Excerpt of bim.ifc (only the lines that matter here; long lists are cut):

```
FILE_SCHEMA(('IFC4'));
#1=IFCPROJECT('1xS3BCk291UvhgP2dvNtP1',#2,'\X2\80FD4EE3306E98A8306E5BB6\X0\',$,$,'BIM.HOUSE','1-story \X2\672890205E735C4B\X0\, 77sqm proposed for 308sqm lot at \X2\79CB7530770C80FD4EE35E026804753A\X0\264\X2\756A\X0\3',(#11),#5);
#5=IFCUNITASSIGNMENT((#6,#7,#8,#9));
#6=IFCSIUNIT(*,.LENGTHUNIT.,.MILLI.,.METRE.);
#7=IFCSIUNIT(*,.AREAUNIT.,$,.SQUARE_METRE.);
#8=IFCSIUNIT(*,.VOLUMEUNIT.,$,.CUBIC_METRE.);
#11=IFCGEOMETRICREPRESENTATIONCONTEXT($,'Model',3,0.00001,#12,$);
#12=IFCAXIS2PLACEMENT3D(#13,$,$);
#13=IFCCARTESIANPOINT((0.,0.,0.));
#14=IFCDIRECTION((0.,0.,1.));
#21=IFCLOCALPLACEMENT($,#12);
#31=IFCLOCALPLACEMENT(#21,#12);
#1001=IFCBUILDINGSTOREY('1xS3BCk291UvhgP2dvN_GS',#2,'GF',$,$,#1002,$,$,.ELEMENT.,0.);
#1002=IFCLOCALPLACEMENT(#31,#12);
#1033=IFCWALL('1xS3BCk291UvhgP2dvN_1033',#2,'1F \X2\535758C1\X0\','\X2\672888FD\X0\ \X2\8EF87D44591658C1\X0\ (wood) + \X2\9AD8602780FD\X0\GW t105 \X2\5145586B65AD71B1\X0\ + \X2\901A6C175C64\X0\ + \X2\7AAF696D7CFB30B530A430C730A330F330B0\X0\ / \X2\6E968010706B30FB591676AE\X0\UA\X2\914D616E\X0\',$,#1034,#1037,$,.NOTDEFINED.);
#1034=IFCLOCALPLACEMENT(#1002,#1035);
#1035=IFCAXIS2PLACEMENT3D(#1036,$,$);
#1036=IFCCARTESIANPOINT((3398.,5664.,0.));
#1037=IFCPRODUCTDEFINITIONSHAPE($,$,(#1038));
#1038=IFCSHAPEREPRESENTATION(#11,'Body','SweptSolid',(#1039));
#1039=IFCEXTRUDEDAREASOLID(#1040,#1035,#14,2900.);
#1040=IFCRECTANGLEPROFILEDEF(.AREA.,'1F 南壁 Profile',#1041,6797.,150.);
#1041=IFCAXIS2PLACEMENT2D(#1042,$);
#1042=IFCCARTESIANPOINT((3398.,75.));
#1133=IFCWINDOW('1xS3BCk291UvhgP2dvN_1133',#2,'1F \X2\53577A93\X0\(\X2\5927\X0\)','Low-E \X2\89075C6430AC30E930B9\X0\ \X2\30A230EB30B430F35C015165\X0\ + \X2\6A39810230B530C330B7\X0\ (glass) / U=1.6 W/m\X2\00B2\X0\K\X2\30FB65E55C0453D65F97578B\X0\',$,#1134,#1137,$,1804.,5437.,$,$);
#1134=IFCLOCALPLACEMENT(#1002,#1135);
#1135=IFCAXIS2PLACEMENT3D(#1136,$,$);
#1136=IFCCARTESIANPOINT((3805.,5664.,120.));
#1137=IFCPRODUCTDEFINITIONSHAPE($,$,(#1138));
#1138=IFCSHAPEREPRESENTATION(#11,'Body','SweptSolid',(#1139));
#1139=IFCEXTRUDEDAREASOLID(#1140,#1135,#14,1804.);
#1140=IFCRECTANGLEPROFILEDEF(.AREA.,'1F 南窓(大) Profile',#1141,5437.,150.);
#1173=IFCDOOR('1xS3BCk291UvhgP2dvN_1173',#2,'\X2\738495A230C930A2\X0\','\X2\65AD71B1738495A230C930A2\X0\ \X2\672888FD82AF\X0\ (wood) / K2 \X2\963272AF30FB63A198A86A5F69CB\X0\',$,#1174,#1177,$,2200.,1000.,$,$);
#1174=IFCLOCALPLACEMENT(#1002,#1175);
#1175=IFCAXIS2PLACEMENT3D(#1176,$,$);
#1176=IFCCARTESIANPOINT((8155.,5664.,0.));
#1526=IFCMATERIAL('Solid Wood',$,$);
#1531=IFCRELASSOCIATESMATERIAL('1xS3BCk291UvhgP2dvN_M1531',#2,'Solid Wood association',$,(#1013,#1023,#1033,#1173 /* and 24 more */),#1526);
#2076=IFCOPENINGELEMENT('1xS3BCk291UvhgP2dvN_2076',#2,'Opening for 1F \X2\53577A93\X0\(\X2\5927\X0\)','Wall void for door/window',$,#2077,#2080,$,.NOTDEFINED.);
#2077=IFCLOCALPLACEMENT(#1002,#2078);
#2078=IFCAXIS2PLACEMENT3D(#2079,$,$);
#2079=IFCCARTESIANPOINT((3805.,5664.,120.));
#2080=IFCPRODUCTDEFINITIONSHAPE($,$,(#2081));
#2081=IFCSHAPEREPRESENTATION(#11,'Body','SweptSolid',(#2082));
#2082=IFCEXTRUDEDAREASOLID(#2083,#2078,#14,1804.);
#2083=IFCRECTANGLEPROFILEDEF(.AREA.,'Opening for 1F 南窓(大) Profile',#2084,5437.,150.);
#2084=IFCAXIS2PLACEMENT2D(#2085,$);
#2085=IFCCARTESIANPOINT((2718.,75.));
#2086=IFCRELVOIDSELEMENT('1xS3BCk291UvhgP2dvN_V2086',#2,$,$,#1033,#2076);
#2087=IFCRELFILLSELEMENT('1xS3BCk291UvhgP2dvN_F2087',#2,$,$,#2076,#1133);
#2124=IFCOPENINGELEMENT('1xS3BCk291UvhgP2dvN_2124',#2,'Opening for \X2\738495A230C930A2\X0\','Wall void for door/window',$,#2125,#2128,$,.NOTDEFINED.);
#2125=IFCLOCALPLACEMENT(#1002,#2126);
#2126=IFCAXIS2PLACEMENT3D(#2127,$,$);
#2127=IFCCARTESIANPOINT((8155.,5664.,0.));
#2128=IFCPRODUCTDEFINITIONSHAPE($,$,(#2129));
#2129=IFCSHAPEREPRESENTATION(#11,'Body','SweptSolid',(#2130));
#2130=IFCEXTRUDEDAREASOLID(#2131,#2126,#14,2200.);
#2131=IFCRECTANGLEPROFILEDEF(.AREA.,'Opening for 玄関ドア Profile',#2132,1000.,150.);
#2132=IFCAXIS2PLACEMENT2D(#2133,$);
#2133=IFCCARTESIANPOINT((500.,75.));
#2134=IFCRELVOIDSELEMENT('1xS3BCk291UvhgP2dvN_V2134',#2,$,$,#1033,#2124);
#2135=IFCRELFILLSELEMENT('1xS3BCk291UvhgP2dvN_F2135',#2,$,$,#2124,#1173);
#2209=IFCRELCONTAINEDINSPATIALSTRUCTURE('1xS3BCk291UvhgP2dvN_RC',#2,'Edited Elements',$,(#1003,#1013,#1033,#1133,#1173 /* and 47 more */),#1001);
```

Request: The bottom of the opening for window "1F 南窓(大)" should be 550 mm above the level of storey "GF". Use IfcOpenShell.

```python
import numpy as np
import ifcopenshell
import ifcopenshell.api.geometry
import ifcopenshell.geom
import ifcopenshell.util.element
import ifcopenshell.util.placement
import ifcopenshell.util.shape
import ifcopenshell.util.unit

model = ifcopenshell.open("bim.ifc")
unit_scale = ifcopenshell.util.unit.calculate_unit_scale(model)

window = model.by_guid("1xS3BCk291UvhgP2dvN_1133")
opening = window.FillsVoids[0].RelatingOpeningElement
storey = ifcopenshell.util.element.get_container(window, ifc_class="IfcBuildingStorey")
level = ifcopenshell.util.placement.get_local_placement(storey.ObjectPlacement)[2, 3]

# The opening's origin need not be at the sill, so measure its lowest point.
shape = ifcopenshell.geom.create_shape(ifcopenshell.geom.settings(), opening)
bottom = ifcopenshell.util.shape.get_shape_bottom_elevation(shape, shape.geometry) / unit_scale
dz = level + 0.55 / unit_scale - bottom

shift = np.array([0.0, 0.0, dz])
# The window is not placed relative to its opening, so move both.
for product in (opening, window):
    matrix = ifcopenshell.util.placement.get_local_placement(product.ObjectPlacement)
    matrix[:3, 3] += shift
    ifcopenshell.api.geometry.edit_object_placement(model, product=product, matrix=matrix, is_si=False)

print(f"moved by {dz * unit_scale:+.3f} m")

model.write("bim_v2.ifc")
```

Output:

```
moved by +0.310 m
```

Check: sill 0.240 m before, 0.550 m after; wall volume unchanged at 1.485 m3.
